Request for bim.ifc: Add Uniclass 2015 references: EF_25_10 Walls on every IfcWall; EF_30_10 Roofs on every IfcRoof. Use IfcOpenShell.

First a look at what the model holds.

```python
import ifcopenshell

model = ifcopenshell.open("bim.ifc")
print(model.schema)
print("classifications:", [c.Name for c in model.by_type("IfcClassification")])
for ifc_class in ("IfcDoor", "IfcRoof", "IfcStair", "IfcWall", "IfcWindow"):
    print(ifc_class, len(model.by_type(ifc_class)))
```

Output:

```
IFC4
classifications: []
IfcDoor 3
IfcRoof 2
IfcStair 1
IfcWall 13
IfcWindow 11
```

```python
import ifcopenshell
import ifcopenshell.api.classification

model = ifcopenshell.open("bim.ifc")

system = ifcopenshell.api.classification.add_classification(model, classification="Uniclass 2015")

codes = {
    "IfcWall": ("EF_25_10", "Walls"),
    "IfcRoof": ("EF_30_10", "Roofs"),
}
for ifc_class, (code, name) in codes.items():
    products = model.by_type(ifc_class)
    ifcopenshell.api.classification.add_reference(
        model, products=products, classification=system, identification=code, name=name
    )
    print(code, len(products))

model.write("bim_updated.ifc")
```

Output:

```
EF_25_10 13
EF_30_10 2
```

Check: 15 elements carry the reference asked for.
